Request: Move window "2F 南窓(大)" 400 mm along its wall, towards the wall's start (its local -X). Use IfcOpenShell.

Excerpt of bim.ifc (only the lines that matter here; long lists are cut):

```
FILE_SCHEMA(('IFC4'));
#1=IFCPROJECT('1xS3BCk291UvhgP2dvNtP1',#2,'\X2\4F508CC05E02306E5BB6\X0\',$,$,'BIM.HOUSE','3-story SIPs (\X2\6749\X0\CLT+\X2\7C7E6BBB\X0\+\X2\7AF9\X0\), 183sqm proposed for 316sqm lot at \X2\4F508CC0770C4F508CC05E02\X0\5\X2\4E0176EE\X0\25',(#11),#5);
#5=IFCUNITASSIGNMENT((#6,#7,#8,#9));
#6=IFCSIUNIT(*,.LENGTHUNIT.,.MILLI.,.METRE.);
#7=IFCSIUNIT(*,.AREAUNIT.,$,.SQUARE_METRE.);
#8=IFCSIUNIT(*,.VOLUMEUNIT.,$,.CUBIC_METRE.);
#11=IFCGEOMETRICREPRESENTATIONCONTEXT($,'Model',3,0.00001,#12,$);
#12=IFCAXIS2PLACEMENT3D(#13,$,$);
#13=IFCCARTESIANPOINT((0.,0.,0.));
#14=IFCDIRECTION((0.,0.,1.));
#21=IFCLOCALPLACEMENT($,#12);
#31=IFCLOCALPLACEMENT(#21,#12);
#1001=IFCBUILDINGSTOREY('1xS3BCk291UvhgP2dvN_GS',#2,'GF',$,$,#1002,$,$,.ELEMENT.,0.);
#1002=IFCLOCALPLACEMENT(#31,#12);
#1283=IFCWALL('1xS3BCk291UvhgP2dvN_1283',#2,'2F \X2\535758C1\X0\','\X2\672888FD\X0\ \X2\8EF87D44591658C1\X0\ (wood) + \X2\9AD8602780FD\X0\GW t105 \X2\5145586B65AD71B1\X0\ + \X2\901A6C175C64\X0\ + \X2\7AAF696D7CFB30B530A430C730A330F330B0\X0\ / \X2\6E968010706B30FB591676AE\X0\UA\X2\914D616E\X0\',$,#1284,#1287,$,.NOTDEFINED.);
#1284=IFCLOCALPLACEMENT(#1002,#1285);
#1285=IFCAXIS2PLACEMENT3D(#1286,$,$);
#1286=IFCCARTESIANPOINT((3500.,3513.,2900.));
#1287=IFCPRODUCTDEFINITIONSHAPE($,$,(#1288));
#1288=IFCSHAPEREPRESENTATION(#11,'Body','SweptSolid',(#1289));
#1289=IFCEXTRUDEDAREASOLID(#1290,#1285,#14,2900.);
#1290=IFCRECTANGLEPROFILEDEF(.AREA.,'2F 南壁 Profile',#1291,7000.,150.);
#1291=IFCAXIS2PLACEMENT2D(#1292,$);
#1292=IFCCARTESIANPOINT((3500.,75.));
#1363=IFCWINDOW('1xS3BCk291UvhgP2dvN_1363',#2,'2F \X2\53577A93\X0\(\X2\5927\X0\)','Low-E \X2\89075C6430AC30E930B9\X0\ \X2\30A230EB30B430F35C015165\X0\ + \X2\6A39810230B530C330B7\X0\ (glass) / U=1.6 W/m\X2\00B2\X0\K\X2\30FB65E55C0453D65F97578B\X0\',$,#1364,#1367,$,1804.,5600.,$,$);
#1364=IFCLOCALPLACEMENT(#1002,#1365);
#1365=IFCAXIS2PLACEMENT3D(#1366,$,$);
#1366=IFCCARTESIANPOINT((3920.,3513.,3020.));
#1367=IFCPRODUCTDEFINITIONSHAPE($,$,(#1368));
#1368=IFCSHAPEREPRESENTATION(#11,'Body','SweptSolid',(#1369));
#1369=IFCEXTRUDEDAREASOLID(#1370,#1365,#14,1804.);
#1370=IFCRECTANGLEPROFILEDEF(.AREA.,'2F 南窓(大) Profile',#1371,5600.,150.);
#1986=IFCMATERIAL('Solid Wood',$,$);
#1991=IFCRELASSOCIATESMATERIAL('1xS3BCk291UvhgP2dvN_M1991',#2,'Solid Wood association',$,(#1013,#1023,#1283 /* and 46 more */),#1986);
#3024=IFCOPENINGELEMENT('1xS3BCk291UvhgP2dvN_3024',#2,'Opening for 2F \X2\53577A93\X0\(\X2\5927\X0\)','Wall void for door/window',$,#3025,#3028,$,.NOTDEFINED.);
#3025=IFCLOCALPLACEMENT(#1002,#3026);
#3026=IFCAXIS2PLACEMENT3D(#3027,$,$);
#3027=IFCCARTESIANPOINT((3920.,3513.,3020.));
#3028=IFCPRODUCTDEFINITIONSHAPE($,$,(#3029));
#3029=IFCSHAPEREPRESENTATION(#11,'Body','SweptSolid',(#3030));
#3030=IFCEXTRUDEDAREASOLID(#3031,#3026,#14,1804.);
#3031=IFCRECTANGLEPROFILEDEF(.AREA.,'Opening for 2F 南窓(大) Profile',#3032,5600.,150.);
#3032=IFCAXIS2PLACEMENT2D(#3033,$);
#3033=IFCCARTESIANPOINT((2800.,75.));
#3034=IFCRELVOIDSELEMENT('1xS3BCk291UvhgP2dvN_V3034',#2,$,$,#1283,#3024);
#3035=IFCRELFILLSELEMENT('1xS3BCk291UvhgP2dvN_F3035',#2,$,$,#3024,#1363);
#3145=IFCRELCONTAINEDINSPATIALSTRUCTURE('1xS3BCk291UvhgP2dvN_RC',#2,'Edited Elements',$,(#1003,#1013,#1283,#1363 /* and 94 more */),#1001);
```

```python
import ifcopenshell
import ifcopenshell.api.geometry
import ifcopenshell.util.placement

model = ifcopenshell.open("bim.ifc")

window = model.by_guid("1xS3BCk291UvhgP2dvN_1363")
opening = window.FillsVoids[0].RelatingOpeningElement
wall = opening.VoidsElements[0].RelatingBuildingElement

wall_matrix = ifcopenshell.util.placement.get_local_placement(wall.ObjectPlacement)
shift = wall_matrix[:3, 0] * -400.0
before = ifcopenshell.util.placement.get_local_placement(window.ObjectPlacement)[:3, 3].copy()

# The window is not placed relative to its opening, so move both.
for product in (opening, window):
    matrix = ifcopenshell.util.placement.get_local_placement(product.ObjectPlacement)
    matrix[:3, 3] += shift
    ifcopenshell.api.geometry.edit_object_placement(model, product=product, matrix=matrix, is_si=False)

after = ifcopenshell.util.placement.get_local_placement(window.ObjectPlacement)[:3, 3]
print("window moved by", (after - before).round(3) + 0.0)

model.write("bim-out.ifc")
```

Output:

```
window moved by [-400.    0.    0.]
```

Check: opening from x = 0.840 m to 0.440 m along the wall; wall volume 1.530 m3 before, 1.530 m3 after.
